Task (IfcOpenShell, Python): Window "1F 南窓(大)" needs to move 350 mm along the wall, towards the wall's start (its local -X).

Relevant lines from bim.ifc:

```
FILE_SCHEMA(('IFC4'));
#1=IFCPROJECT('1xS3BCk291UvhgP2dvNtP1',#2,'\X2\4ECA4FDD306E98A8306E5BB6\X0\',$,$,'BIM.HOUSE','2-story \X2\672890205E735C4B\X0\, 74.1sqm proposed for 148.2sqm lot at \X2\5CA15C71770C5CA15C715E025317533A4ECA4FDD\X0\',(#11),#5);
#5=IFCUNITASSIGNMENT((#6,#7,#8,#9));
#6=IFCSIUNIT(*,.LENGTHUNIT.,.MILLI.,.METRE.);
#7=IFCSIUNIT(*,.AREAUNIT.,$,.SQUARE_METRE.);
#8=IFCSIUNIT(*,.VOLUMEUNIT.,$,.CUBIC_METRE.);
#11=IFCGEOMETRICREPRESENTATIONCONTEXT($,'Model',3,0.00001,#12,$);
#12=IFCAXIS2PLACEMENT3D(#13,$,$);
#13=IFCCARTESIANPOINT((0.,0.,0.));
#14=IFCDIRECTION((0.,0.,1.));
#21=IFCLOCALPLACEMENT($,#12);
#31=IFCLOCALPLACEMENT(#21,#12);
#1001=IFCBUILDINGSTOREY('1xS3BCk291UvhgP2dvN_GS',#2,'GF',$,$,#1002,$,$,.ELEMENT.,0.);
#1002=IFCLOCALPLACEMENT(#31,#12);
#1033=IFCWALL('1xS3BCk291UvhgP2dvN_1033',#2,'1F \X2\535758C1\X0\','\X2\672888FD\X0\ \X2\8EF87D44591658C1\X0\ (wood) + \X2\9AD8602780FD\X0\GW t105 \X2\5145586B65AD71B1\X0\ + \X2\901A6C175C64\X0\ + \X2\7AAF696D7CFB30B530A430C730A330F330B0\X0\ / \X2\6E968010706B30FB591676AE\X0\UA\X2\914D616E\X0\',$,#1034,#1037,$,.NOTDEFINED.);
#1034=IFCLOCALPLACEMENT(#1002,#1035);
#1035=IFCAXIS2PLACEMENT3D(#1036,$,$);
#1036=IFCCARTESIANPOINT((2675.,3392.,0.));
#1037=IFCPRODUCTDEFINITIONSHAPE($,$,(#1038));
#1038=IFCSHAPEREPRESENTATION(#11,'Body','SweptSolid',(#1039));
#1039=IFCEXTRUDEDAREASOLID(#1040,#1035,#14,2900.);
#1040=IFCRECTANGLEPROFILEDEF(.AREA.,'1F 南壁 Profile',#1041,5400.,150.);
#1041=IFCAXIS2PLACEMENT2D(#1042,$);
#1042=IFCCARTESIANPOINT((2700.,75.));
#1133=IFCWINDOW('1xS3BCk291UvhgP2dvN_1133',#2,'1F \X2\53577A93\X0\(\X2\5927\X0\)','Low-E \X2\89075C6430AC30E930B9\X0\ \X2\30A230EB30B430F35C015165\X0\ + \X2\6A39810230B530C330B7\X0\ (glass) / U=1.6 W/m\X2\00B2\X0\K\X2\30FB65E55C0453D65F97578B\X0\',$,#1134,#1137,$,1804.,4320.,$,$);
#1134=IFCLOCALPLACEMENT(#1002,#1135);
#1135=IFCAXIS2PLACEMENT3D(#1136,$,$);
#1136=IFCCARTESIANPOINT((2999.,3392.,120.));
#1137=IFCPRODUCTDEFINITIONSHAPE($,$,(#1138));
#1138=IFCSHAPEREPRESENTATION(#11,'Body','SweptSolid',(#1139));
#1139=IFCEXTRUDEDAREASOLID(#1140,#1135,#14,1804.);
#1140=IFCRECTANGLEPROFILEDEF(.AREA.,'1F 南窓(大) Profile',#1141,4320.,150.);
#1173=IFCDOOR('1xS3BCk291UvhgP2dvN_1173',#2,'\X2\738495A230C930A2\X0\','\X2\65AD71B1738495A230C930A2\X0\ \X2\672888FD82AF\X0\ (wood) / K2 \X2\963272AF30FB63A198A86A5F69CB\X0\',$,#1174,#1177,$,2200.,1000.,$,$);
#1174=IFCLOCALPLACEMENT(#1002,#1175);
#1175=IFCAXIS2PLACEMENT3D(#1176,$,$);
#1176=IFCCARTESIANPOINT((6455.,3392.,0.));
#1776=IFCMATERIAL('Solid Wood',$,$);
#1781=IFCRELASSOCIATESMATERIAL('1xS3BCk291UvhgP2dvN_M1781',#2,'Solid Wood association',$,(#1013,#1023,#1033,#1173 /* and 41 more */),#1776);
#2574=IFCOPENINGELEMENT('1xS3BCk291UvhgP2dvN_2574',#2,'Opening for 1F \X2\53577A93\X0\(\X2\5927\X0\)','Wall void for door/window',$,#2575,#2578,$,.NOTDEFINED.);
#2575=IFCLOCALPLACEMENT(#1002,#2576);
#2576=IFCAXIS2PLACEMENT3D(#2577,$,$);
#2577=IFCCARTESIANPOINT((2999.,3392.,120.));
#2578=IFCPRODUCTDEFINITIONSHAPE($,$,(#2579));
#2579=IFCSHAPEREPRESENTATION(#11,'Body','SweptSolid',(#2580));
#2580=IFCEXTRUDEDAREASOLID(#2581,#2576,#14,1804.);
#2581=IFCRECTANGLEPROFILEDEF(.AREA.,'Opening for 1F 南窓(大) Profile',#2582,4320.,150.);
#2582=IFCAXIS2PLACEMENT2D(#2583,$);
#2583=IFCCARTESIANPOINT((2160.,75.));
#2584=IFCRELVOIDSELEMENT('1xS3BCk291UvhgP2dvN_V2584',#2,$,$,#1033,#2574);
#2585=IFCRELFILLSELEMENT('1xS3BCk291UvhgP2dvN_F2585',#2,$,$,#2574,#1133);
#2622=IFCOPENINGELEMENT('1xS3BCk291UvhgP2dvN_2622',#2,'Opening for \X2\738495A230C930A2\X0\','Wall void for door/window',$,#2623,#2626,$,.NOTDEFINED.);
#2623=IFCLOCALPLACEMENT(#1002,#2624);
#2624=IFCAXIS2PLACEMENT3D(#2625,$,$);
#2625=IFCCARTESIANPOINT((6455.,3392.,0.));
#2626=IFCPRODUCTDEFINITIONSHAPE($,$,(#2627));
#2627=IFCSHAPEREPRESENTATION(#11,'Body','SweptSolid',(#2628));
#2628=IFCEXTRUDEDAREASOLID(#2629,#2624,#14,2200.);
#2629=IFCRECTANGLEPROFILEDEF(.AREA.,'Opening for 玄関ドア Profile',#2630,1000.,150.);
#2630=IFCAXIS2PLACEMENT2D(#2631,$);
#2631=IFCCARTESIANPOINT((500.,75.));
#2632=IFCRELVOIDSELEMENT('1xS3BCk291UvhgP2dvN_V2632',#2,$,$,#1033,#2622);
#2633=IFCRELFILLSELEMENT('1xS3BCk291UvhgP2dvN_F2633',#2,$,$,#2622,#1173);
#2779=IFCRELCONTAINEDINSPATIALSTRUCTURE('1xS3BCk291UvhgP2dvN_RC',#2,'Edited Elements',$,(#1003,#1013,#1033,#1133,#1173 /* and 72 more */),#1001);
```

```python
import ifcopenshell
import ifcopenshell.api.geometry
import ifcopenshell.util.placement
import ifcopenshell.util.unit

model = ifcopenshell.open("bim.ifc")
unit_scale = ifcopenshell.util.unit.calculate_unit_scale(model)

window = model.by_id(1133)
opening = window.FillsVoids[0].RelatingOpeningElement
wall = opening.VoidsElements[0].RelatingBuildingElement

wall_matrix = ifcopenshell.util.placement.get_local_placement(wall.ObjectPlacement)
shift = wall_matrix[:3, 0] * -0.35 / unit_scale
before = ifcopenshell.util.placement.get_local_placement(window.ObjectPlacement)[:3, 3].copy()

# The window is not placed relative to its opening, so move both.
for product in (opening, window):
    matrix = ifcopenshell.util.placement.get_local_placement(product.ObjectPlacement)
    matrix[:3, 3] += shift
    ifcopenshell.api.geometry.edit_object_placement(model, product=product, matrix=matrix, is_si=False)

after = ifcopenshell.util.placement.get_local_placement(window.ObjectPlacement)[:3, 3]
print("window moved by", (after - before).round(3) + 0.0)

model.write("bim_v2.ifc")
```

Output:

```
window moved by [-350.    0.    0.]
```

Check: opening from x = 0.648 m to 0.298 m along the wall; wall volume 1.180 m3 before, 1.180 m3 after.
